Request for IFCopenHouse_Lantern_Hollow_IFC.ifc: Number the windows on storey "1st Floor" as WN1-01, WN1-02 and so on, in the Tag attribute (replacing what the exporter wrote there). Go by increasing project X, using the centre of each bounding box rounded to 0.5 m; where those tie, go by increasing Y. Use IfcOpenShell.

First a look at what the model holds.

```python
import ifcopenshell
import ifcopenshell.util.element
import ifcopenshell.util.placement

model = ifcopenshell.open("IFCopenHouse_Lantern_Hollow_IFC.ifc")
print(model.schema)
storey = next(s for s in model.by_type("IfcBuildingStorey") if s.Name == "1st Floor")
windows = [e for e in ifcopenshell.util.element.get_decomposition(storey) if e.is_a("IfcWindow")]
for e in sorted(windows, key=lambda e: e.id()):
    origin = ifcopenshell.util.placement.get_local_placement(e.ObjectPlacement)[:3, 3]
    print(e.id(), e.Tag, e.Name, origin.round(2) + 0.0, sep=" | ")
```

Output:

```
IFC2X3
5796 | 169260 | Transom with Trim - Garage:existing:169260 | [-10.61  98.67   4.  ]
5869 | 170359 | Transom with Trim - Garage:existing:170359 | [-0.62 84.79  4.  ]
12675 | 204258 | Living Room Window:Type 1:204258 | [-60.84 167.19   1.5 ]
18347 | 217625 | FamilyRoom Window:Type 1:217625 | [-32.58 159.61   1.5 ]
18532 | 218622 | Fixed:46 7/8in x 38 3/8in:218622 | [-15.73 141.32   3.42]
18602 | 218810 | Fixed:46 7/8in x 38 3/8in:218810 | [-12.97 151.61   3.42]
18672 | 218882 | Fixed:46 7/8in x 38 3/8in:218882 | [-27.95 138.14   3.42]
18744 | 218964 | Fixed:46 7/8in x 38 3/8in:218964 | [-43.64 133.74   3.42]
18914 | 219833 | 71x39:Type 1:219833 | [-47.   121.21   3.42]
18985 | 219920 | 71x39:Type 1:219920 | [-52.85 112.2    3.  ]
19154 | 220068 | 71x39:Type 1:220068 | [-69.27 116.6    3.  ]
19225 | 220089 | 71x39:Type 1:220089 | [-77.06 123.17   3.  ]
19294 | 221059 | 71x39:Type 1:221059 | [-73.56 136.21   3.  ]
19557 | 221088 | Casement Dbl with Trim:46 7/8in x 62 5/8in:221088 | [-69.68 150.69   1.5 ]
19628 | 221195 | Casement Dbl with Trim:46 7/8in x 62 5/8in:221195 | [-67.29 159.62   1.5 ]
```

```python
import ifcopenshell
import ifcopenshell.geom
import ifcopenshell.util.element
import ifcopenshell.util.shape

model = ifcopenshell.open("IFCopenHouse_Lantern_Hollow_IFC.ifc")
settings = ifcopenshell.geom.settings()
settings.set("use-world-coords", True)


def centre(element):
    shape = ifcopenshell.geom.create_shape(settings, element)
    return ifcopenshell.util.shape.get_bbox_centroid(shape.geometry)


storey = next(s for s in model.by_type("IfcBuildingStorey") if s.Name == "1st Floor")
windows = [e for e in ifcopenshell.util.element.get_decomposition(storey) if e.is_a("IfcWindow")]

# Insertion points can sit at a corner or the storey origin, so sort by the geometry (in metres).
centres = {e: centre(e) for e in windows}
windows.sort(key=lambda e: (round(centres[e][0] / 0.5), centres[e][1]))

for i, e in enumerate(windows, start=1):
    number = f"WN1-{i:02d}"
    e.Tag = number
    print(e.id(), number)

model.write("IFCopenHouse_Lantern_Hollow_IFC_updated.ifc")
```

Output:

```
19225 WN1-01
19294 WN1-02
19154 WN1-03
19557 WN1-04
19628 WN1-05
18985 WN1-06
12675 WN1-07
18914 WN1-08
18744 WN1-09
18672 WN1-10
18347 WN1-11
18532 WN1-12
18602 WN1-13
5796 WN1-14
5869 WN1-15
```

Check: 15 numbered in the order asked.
